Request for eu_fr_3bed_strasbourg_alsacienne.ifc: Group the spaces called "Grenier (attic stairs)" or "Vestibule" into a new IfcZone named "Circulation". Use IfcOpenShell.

First a look at what the model holds.

```python
import ifcopenshell

model = ifcopenshell.open("eu_fr_3bed_strasbourg_alsacienne.ifc")
print(model.schema)
seen = {}
for space in model.by_type("IfcSpace"):
    seen[space.LongName] = seen.get(space.LongName, 0) + 1
for name, count in sorted(seen.items(), key=str):
    print(count, "x", name)
print("zones:", [z.Name for z in model.by_type("IfcZone")][:20])
```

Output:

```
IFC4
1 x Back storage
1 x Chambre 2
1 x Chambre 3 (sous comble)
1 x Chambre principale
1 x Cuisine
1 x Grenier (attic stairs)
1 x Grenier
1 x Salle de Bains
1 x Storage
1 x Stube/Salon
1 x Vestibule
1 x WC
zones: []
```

```python
import ifcopenshell
import ifcopenshell.api.group
import ifcopenshell.api.root

model = ifcopenshell.open("eu_fr_3bed_strasbourg_alsacienne.ifc")

names = {"Grenier (attic stairs)", "Vestibule"}
spaces = [s for s in model.by_type("IfcSpace") if s.LongName in names]

zone = ifcopenshell.api.root.create_entity(model, ifc_class="IfcZone", name="Circulation")
ifcopenshell.api.group.assign_group(model, products=spaces, group=zone)
print(len(spaces), "spaces in", zone.Name)

model.write("eu_fr_3bed_strasbourg_alsacienne_edited.ifc")
```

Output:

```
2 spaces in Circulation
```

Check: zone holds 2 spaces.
